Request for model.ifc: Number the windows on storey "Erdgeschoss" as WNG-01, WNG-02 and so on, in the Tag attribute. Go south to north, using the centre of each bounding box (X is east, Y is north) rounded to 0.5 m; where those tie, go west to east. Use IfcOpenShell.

First a look at what the model holds.

```python
import ifcopenshell
import ifcopenshell.util.element
import ifcopenshell.util.placement

model = ifcopenshell.open("model.ifc")
print(model.schema)
storey = next(s for s in model.by_type("IfcBuildingStorey") if s.Name == "Erdgeschoss")
windows = [e for e in ifcopenshell.util.element.get_decomposition(storey) if e.is_a("IfcWindow")]
for e in sorted(windows, key=lambda e: e.id()):
    origin = ifcopenshell.util.placement.get_local_placement(e.ObjectPlacement)[:3, 3]
    print(e.id(), e.Tag, e.Name, origin.round(2) + 0.0, sep=" | ")
```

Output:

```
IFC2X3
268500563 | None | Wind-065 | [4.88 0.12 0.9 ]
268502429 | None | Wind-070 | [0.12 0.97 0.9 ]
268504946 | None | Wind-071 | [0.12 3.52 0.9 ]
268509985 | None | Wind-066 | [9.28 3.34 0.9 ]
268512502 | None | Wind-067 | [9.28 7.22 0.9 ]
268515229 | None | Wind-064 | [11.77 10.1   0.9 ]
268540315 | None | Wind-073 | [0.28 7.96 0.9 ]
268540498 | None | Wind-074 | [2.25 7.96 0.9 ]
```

```python
import ifcopenshell
import ifcopenshell.geom
import ifcopenshell.util.element
import ifcopenshell.util.shape

model = ifcopenshell.open("model.ifc")
settings = ifcopenshell.geom.settings()
settings.set("use-world-coords", True)


def centre(element):
    shape = ifcopenshell.geom.create_shape(settings, element)
    return ifcopenshell.util.shape.get_bbox_centroid(shape.geometry)


storey = next(s for s in model.by_type("IfcBuildingStorey") if s.Name == "Erdgeschoss")
windows = [e for e in ifcopenshell.util.element.get_decomposition(storey) if e.is_a("IfcWindow")]

# Insertion points can sit at a corner or the storey origin, so sort by the geometry (in metres).
centres = {e: centre(e) for e in windows}
windows.sort(key=lambda e: (round(centres[e][1] / 0.5), centres[e][0]))

for i, e in enumerate(windows, start=1):
    number = f"WNG-{i:02d}"
    e.Tag = number
    print(e.id(), number)

model.write("model-out.ifc")
```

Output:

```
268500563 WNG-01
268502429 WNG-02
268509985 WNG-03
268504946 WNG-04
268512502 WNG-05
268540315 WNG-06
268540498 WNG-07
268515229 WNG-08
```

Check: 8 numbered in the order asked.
